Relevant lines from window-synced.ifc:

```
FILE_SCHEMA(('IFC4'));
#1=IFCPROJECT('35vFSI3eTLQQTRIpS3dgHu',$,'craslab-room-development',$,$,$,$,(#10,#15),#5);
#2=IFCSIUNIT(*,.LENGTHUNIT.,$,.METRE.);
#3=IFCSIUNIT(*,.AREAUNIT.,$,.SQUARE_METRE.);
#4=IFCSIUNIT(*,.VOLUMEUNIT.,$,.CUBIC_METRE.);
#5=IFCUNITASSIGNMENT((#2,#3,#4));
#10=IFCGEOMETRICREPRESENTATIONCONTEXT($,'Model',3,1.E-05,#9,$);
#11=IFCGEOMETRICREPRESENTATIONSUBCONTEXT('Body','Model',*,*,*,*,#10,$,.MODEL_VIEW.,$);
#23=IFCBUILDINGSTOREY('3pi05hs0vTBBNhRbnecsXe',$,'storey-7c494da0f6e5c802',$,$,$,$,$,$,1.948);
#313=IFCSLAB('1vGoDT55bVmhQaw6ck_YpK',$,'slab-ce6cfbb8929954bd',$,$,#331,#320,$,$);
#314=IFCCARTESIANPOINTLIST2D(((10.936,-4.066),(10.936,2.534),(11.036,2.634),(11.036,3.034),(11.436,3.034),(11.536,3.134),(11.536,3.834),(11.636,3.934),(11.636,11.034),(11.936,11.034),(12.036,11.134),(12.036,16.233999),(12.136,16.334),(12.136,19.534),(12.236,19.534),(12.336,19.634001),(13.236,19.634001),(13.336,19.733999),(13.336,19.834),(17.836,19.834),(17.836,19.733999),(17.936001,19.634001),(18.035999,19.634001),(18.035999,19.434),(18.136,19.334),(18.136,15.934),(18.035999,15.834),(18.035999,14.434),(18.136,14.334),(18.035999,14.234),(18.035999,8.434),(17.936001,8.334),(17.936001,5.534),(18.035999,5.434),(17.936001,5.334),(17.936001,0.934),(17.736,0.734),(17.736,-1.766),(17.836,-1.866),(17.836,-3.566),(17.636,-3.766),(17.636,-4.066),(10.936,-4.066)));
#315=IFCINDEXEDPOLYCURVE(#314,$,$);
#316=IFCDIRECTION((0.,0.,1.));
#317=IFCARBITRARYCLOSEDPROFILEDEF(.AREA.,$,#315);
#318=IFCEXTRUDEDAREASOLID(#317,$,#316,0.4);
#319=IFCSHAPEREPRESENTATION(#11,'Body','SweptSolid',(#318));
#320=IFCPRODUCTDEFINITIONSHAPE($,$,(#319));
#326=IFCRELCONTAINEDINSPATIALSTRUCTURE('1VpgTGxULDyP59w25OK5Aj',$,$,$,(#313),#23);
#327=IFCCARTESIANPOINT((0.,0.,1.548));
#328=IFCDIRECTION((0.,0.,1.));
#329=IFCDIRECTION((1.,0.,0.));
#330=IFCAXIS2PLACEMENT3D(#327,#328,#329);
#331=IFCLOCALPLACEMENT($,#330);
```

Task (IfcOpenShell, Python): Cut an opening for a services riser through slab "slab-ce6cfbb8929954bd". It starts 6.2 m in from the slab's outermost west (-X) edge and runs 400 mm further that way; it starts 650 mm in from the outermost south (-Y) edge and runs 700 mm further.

```python
import numpy as np
import ifcopenshell
import ifcopenshell.api.feature
import ifcopenshell.api.geometry
import ifcopenshell.api.root
import ifcopenshell.geom
import ifcopenshell.util.placement
import ifcopenshell.util.representation
import ifcopenshell.util.shape
import ifcopenshell.util.unit

model = ifcopenshell.open("window-synced.ifc")
unit_scale = ifcopenshell.util.unit.calculate_unit_scale(model)
settings = ifcopenshell.geom.settings()


def volume(element):
    """Net volume in cubic metres, openings subtracted."""
    shape = ifcopenshell.geom.create_shape(settings, element)
    return ifcopenshell.util.shape.get_volume(shape.geometry)


slab = model.by_id(313)
before = volume(slab)

# Extent in the slab's own axes, in metres. The edges named are its -X and -Y sides.
slab_shape = ifcopenshell.geom.create_shape(settings, slab)
vertices = ifcopenshell.util.shape.get_vertices(slab_shape.geometry)
x_min, y_min, bottom = vertices.min(axis=0)
top = vertices[:, 2].max()

opening = ifcopenshell.api.root.create_entity(model, ifc_class="IfcOpeningElement", name="Services riser opening", predefined_type="OPENING")
context = ifcopenshell.util.representation.get_context(model, "Model", "Body", "MODEL_VIEW")
width, depth = 0.4, 0.7
outline = [(0.0, 0.0), (width, 0.0), (width, depth), (0.0, depth), (0.0, 0.0)]
# Overshoot both faces by 50 mm so the cut is clean.
shape = ifcopenshell.api.geometry.add_slab_representation(
    model, context=context, depth=top - bottom + 0.1, polyline=outline
)
ifcopenshell.api.geometry.assign_representation(model, product=opening, representation=shape)

matrix = ifcopenshell.util.placement.get_local_placement(slab.ObjectPlacement)
matrix[:, 3] = matrix @ np.append(np.array([x_min + 6.2, y_min + 0.65, bottom - 0.05]) / unit_scale, 1.0)
ifcopenshell.api.geometry.edit_object_placement(model, product=opening, matrix=matrix, is_si=False)
ifcopenshell.api.feature.add_feature(model, feature=opening, element=slab)

after = volume(slab)

print(f"slab volume {before:.3f} -> {after:.3f} m3")

model.write("window-synced_edited.ifc")
```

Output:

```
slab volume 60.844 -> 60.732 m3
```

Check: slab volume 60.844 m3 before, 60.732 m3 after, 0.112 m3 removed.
